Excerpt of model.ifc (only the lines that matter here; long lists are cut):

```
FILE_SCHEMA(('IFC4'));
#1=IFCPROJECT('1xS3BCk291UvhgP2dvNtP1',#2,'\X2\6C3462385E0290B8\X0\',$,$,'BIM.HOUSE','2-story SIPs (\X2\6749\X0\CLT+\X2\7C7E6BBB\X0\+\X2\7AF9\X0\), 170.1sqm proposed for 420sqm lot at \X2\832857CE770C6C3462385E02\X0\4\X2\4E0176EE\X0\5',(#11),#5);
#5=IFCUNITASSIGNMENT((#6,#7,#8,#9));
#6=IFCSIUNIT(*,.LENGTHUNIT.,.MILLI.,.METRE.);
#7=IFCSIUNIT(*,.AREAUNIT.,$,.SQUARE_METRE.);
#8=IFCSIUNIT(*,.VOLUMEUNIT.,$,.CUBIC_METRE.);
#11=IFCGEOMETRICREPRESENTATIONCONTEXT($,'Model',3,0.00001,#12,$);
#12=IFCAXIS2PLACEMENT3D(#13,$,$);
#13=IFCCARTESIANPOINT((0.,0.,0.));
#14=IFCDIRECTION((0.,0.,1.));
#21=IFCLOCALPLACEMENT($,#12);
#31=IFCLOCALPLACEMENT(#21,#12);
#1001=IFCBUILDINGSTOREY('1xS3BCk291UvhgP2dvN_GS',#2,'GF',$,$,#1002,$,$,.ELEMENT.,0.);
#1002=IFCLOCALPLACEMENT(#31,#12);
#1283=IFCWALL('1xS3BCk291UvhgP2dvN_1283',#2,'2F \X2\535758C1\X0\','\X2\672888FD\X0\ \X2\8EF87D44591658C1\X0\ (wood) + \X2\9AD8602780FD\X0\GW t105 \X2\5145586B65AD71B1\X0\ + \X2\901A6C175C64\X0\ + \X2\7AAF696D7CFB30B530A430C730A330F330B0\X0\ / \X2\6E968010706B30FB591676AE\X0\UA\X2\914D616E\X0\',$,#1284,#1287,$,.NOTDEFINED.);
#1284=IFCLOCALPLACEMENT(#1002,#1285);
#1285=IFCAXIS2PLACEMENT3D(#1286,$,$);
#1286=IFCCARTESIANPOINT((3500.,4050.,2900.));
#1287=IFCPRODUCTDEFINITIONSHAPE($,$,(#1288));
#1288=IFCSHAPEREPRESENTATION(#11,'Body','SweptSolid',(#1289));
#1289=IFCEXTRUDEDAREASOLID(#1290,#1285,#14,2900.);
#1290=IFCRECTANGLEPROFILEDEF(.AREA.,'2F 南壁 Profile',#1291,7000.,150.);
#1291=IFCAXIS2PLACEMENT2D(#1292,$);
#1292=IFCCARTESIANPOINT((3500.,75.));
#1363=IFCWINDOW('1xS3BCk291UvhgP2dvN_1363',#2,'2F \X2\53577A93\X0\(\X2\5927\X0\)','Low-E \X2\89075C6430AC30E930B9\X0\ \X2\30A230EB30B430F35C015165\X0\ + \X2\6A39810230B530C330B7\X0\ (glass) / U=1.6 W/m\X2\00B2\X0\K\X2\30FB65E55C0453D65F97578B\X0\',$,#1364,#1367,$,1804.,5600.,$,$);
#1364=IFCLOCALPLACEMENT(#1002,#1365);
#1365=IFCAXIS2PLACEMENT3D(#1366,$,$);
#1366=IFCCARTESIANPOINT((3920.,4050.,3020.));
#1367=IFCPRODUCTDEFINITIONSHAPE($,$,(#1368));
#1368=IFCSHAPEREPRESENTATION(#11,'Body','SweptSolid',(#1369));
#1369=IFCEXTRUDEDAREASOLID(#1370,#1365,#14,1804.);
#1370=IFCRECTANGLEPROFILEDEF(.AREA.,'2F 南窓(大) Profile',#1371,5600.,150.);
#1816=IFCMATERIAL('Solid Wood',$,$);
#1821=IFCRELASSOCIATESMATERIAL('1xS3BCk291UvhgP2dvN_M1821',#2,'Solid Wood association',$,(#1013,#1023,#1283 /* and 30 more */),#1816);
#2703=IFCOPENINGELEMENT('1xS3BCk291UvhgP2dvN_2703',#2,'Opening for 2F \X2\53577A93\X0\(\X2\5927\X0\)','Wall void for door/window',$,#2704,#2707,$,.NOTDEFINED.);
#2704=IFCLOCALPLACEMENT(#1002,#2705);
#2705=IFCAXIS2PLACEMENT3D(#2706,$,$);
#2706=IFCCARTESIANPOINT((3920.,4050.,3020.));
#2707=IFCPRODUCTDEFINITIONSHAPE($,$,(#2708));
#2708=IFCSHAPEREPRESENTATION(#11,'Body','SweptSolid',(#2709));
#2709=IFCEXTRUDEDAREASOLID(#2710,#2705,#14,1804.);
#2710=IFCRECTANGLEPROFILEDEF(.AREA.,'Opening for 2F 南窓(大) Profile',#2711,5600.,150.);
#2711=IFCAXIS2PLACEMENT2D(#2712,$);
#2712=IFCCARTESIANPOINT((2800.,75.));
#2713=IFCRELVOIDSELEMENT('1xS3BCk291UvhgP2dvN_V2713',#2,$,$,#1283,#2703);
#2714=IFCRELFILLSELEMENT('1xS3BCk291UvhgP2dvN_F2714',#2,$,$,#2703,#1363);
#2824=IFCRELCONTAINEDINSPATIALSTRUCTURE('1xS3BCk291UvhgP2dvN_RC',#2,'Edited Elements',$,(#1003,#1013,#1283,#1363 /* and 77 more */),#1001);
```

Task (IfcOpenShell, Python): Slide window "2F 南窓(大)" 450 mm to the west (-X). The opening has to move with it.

```python
import ifcopenshell
import ifcopenshell.api.geometry
import ifcopenshell.util.placement
import ifcopenshell.util.unit

model = ifcopenshell.open("model.ifc")
unit_scale = ifcopenshell.util.unit.calculate_unit_scale(model)

window = model.by_guid("1xS3BCk291UvhgP2dvN_1363")
opening = window.FillsVoids[0].RelatingOpeningElement
wall = opening.VoidsElements[0].RelatingBuildingElement

wall_matrix = ifcopenshell.util.placement.get_local_placement(wall.ObjectPlacement)
shift = wall_matrix[:3, 0] * -0.45 / unit_scale
before = ifcopenshell.util.placement.get_local_placement(window.ObjectPlacement)[:3, 3].copy()

# The window is not placed relative to its opening, so move both.
for product in (opening, window):
    matrix = ifcopenshell.util.placement.get_local_placement(product.ObjectPlacement)
    matrix[:3, 3] += shift
    ifcopenshell.api.geometry.edit_object_placement(model, product=product, matrix=matrix, is_si=False)

after = ifcopenshell.util.placement.get_local_placement(window.ObjectPlacement)[:3, 3]
print("window moved by", (after - before).round(3) + 0.0)

model.write("model_edited.ifc")
```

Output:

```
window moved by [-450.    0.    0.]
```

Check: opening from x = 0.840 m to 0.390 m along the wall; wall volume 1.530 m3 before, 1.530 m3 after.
